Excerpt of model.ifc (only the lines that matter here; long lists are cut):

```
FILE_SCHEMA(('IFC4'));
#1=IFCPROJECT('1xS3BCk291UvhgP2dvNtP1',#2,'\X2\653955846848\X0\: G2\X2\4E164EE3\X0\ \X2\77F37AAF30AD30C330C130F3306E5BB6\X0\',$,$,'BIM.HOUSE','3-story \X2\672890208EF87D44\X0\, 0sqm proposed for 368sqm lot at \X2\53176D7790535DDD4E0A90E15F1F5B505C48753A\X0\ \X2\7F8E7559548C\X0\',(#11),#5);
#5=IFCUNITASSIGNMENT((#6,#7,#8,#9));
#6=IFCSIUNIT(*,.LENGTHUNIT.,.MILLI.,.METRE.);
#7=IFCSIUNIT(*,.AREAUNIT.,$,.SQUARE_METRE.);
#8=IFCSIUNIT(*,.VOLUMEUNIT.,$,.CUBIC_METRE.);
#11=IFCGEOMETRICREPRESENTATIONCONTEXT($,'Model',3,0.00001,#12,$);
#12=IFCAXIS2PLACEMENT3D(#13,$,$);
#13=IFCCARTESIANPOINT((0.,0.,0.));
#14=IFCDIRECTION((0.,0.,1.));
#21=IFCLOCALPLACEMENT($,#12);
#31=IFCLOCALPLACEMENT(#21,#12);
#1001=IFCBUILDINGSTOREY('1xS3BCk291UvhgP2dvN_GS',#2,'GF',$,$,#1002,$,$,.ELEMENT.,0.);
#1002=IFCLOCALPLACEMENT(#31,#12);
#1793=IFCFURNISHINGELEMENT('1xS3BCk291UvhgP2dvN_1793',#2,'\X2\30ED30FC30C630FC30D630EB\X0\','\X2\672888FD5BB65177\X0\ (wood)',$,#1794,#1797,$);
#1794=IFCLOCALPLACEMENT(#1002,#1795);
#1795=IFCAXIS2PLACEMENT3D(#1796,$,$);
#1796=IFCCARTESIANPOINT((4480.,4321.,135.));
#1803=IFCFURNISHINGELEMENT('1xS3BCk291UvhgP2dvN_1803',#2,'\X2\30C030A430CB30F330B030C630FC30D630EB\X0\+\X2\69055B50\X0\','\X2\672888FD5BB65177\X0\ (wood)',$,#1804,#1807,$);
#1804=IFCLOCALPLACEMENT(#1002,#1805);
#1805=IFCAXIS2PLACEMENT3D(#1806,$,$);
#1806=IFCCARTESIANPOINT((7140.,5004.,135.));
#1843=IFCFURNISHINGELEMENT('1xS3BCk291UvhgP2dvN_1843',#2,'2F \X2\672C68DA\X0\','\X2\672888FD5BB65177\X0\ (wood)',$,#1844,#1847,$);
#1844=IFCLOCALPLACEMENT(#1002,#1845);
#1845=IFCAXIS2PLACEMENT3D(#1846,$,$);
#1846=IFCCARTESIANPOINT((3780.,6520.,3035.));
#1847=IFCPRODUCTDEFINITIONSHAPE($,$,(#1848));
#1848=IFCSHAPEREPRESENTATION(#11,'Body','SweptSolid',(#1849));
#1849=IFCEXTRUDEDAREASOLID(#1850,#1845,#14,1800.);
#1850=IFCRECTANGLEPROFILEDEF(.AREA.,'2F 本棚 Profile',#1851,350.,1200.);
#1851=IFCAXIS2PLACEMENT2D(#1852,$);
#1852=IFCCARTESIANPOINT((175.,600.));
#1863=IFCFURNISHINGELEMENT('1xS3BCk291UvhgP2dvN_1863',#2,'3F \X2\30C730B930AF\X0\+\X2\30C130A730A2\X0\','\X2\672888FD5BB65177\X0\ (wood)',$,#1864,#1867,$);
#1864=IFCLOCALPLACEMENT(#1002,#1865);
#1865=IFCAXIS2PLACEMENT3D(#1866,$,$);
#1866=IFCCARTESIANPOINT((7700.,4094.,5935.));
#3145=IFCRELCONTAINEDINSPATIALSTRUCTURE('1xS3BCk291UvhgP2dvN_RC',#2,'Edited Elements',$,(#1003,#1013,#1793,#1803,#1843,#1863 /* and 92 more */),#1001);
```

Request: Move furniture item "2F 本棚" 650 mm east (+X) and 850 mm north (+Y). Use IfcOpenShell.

```python
import ifcopenshell
import ifcopenshell.api.geometry
import ifcopenshell.util.placement

model = ifcopenshell.open("model.ifc")

item = model.by_guid("1xS3BCk291UvhgP2dvN_1843")
matrix = ifcopenshell.util.placement.get_local_placement(item.ObjectPlacement)
matrix[0, 3] += 650.0
matrix[1, 3] += 850.0
ifcopenshell.api.geometry.edit_object_placement(model, product=item, matrix=matrix, is_si=False)

print(ifcopenshell.util.placement.get_local_placement(item.ObjectPlacement).round(3) + 0.0)

model.write("model_rev.ifc")
```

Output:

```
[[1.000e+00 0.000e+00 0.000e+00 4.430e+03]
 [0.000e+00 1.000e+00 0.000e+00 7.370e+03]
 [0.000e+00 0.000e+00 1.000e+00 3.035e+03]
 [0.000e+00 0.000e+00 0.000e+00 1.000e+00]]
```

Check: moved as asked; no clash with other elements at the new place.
